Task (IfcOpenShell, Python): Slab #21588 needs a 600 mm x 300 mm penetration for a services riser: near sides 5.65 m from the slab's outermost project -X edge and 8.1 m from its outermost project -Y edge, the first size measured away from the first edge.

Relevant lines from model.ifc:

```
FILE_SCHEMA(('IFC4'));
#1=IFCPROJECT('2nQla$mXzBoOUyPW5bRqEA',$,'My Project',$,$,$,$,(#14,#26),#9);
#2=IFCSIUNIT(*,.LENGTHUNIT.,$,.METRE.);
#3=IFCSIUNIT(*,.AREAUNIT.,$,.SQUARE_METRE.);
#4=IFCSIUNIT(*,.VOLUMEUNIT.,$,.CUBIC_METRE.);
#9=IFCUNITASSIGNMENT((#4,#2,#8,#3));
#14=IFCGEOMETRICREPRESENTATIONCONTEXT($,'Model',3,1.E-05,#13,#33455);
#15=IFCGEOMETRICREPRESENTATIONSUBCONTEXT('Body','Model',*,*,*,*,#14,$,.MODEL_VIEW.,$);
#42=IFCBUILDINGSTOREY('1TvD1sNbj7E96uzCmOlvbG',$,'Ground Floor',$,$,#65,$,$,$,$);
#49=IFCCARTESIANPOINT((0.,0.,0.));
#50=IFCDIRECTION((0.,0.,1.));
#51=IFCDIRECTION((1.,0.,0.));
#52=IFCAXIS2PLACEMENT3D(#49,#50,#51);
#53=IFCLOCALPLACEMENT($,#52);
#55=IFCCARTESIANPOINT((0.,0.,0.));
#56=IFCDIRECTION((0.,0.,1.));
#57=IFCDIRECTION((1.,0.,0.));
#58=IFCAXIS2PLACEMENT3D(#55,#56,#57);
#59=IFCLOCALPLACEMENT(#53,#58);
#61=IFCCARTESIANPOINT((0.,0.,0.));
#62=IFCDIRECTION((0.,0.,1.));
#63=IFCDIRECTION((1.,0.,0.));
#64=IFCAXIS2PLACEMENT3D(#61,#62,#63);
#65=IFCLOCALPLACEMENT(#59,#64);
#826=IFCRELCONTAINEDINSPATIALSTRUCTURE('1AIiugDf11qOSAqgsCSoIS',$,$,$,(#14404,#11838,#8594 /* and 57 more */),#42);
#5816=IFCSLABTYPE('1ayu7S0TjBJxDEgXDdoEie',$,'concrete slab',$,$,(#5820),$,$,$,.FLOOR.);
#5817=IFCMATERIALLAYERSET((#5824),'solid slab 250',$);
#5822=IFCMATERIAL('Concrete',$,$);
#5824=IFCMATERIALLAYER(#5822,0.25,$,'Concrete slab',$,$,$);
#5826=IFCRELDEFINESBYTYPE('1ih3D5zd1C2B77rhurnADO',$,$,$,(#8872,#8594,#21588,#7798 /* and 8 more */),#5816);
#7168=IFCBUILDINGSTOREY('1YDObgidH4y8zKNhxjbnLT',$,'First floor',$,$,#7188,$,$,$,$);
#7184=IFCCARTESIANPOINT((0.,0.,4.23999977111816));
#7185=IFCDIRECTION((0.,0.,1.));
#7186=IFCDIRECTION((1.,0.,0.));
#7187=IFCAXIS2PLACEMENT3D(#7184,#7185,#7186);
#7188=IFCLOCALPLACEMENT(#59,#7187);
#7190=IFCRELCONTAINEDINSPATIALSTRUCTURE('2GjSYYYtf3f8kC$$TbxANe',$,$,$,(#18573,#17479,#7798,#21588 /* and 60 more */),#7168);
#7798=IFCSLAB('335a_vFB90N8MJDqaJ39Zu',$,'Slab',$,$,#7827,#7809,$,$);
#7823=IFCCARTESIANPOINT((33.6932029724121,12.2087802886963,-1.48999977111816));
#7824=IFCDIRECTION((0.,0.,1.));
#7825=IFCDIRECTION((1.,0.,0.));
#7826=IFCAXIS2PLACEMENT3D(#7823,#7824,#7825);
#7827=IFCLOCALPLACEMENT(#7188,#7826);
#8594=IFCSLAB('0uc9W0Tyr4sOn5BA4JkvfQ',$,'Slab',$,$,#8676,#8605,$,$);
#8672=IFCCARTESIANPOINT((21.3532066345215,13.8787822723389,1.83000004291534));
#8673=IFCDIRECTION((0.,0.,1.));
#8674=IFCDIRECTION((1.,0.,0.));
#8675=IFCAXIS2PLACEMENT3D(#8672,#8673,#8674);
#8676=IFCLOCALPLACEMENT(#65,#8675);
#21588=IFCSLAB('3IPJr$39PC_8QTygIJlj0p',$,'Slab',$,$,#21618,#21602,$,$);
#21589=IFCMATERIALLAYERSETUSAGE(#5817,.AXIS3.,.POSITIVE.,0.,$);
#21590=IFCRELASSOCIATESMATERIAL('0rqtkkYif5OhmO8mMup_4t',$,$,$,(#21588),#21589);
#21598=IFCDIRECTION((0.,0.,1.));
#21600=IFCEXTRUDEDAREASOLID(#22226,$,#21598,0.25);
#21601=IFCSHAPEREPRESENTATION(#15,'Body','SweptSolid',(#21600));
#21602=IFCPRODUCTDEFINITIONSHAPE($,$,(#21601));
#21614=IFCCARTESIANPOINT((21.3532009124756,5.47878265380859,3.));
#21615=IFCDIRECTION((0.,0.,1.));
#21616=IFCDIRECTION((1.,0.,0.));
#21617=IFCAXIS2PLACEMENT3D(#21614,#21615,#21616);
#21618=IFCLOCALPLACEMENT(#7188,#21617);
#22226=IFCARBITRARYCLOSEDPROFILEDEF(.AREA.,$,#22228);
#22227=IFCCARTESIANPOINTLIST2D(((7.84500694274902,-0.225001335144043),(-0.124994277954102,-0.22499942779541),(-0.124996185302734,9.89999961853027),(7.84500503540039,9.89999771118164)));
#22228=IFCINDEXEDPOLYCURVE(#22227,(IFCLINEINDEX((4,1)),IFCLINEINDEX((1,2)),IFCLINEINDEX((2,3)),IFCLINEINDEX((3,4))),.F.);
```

```python
import numpy as np
import ifcopenshell
import ifcopenshell.api.feature
import ifcopenshell.api.geometry
import ifcopenshell.api.root
import ifcopenshell.geom
import ifcopenshell.util.placement
import ifcopenshell.util.representation
import ifcopenshell.util.shape
import ifcopenshell.util.unit

model = ifcopenshell.open("model.ifc")
unit_scale = ifcopenshell.util.unit.calculate_unit_scale(model)
settings = ifcopenshell.geom.settings()


def volume(element):
    """Net volume in cubic metres, openings subtracted."""
    shape = ifcopenshell.geom.create_shape(settings, element)
    return ifcopenshell.util.shape.get_volume(shape.geometry)


slab = model.by_id(21588)
before = volume(slab)

# Extent in the slab's own axes, in metres. The edges named are its -X and -Y sides.
slab_shape = ifcopenshell.geom.create_shape(settings, slab)
vertices = ifcopenshell.util.shape.get_vertices(slab_shape.geometry)
x_min, y_min, bottom = vertices.min(axis=0)
top = vertices[:, 2].max()

opening = ifcopenshell.api.root.create_entity(model, ifc_class="IfcOpeningElement", name="Services riser opening", predefined_type="OPENING")
context = ifcopenshell.util.representation.get_context(model, "Model", "Body", "MODEL_VIEW")
width, depth = 0.6, 0.3
outline = [(0.0, 0.0), (width, 0.0), (width, depth), (0.0, depth), (0.0, 0.0)]
# Overshoot both faces by 50 mm so the cut is clean.
shape = ifcopenshell.api.geometry.add_slab_representation(
    model, context=context, depth=top - bottom + 0.1, polyline=outline
)
ifcopenshell.api.geometry.assign_representation(model, product=opening, representation=shape)

matrix = ifcopenshell.util.placement.get_local_placement(slab.ObjectPlacement)
matrix[:, 3] = matrix @ np.append(np.array([x_min + 5.65, y_min + 8.1, bottom - 0.05]) / unit_scale, 1.0)
ifcopenshell.api.geometry.edit_object_placement(model, product=opening, matrix=matrix, is_si=False)
ifcopenshell.api.feature.add_feature(model, feature=opening, element=slab)

after = volume(slab)

print(f"slab volume {before:.3f} -> {after:.3f} m3")

model.write("model_rev.ifc")
```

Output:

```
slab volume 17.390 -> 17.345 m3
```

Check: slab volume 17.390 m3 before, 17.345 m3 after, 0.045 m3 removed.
